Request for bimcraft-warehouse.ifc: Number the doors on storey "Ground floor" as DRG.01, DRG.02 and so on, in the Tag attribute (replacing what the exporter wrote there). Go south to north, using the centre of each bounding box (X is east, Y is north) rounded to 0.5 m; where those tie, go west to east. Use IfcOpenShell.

First a look at what the model holds.

```python
import ifcopenshell
import ifcopenshell.util.element
import ifcopenshell.util.placement

model = ifcopenshell.open("bimcraft-warehouse.ifc")
print(model.schema)
storey = next(s for s in model.by_type("IfcBuildingStorey") if s.Name == "Ground floor")
doors = [e for e in ifcopenshell.util.element.get_decomposition(storey) if e.is_a("IfcDoor")]
for e in sorted(doors, key=lambda e: e.id()):
    origin = ifcopenshell.util.placement.get_local_placement(e.ObjectPlacement)[:3, 3]
    print(e.id(), e.Tag, e.Name, origin.round(2) + 0.0, sep=" | ")
```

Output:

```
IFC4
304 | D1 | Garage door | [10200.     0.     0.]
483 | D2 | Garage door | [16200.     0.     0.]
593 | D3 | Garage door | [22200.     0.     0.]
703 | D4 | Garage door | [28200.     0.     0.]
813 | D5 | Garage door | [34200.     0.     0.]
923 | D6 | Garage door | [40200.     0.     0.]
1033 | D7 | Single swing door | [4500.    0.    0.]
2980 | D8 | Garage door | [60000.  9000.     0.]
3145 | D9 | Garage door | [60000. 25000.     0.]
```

```python
import ifcopenshell
import ifcopenshell.geom
import ifcopenshell.util.element
import ifcopenshell.util.shape

model = ifcopenshell.open("bimcraft-warehouse.ifc")
settings = ifcopenshell.geom.settings()
settings.set("use-world-coords", True)


def centre(element):
    shape = ifcopenshell.geom.create_shape(settings, element)
    return ifcopenshell.util.shape.get_bbox_centroid(shape.geometry)


storey = next(s for s in model.by_type("IfcBuildingStorey") if s.Name == "Ground floor")
doors = [e for e in ifcopenshell.util.element.get_decomposition(storey) if e.is_a("IfcDoor")]

# Insertion points can sit at a corner or the storey origin, so sort by the geometry (in metres).
centres = {e: centre(e) for e in doors}
doors.sort(key=lambda e: (round(centres[e][1] / 0.5), centres[e][0]))

for i, e in enumerate(doors, start=1):
    number = f"DRG.{i:02d}"
    e.Tag = number
    print(e.id(), number)

model.write("bimcraft-warehouse_rev.ifc")
```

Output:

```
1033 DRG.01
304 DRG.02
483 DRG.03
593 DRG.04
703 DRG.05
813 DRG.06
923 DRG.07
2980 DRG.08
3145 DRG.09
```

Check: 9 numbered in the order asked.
